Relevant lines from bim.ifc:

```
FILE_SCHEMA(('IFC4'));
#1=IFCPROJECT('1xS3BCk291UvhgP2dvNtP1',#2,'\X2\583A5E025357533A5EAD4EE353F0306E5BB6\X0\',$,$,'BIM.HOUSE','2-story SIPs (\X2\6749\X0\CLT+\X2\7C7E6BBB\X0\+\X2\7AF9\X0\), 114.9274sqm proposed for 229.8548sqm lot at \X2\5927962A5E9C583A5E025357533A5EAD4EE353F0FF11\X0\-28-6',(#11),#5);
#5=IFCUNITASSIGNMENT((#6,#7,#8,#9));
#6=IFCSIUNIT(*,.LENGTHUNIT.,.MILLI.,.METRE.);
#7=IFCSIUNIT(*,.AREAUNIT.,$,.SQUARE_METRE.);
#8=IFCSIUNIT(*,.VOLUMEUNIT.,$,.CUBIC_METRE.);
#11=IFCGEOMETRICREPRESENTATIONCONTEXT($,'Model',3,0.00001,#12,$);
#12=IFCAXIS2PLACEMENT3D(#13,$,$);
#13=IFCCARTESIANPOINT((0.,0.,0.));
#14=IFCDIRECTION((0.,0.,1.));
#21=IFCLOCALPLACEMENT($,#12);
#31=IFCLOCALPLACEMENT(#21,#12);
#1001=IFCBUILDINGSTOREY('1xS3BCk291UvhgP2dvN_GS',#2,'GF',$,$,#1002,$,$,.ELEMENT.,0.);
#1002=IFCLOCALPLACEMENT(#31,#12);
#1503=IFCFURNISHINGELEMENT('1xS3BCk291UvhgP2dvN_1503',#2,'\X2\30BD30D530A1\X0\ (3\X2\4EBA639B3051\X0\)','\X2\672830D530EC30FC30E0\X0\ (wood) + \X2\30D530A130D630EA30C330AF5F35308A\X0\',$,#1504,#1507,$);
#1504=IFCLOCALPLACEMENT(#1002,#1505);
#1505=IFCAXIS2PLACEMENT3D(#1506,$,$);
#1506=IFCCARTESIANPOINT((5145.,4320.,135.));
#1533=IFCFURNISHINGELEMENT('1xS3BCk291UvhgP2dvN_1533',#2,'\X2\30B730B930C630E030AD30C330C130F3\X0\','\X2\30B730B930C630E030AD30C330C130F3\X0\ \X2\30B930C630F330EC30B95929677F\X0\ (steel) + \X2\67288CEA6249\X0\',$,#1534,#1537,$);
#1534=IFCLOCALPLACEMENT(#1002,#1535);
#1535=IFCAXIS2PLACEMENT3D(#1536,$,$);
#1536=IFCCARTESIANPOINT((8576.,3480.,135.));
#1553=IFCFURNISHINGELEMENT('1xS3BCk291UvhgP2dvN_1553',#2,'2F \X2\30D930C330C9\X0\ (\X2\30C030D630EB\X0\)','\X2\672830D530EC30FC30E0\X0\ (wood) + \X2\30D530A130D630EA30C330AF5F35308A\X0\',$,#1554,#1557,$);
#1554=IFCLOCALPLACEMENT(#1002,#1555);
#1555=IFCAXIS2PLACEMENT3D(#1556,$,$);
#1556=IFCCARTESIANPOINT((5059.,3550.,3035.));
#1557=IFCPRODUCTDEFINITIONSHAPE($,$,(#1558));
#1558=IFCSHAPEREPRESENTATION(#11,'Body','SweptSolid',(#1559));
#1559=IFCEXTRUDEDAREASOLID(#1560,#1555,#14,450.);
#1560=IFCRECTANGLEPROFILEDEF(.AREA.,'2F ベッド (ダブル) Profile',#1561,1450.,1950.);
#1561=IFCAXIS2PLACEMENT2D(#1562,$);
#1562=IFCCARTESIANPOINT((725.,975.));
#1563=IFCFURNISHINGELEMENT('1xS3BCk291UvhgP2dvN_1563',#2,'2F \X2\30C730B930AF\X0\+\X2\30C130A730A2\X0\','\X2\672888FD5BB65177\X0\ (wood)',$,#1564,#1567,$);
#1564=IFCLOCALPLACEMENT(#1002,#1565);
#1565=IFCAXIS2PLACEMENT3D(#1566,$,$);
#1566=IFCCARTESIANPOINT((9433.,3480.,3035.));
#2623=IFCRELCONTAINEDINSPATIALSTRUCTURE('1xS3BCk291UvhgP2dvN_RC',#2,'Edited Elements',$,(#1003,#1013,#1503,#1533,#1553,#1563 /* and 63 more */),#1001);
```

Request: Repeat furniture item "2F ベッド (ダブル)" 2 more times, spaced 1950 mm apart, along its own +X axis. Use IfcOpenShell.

```python
import ifcopenshell
import ifcopenshell.api.geometry
import ifcopenshell.api.root
import ifcopenshell.util.element
import ifcopenshell.util.placement

model = ifcopenshell.open("bim.ifc")


def reuse_history(source, copy):
    """copy_class also copies each property set's owner history, people and application; keep the originals."""
    for rel in copy.IsDefinedBy:
        if rel.is_a("IfcRelDefinesByProperties") and (history := rel.RelatingPropertyDefinition.OwnerHistory):
            rel.RelatingPropertyDefinition.OwnerHistory = source.OwnerHistory
            ifcopenshell.util.element.remove_deep2(model, history)


source = model.by_guid("1xS3BCk291UvhgP2dvN_1553")
base = ifcopenshell.util.placement.get_local_placement(source.ObjectPlacement)
step = base[:3, 0] * 1950.0

for i in range(1, 3):
    copy = ifcopenshell.api.root.copy_class(model, product=source)
    copy.Representation = ifcopenshell.util.element.copy_deep(
        model, source.Representation, exclude=["IfcGeometricRepresentationContext", "IfcRepresentationMap"]
    )
    reuse_history(source, copy)
    matrix = base.copy()
    matrix[:3, 3] += i * step
    print("added at", matrix[:3, 3].round(3) + 0.0)
    ifcopenshell.api.geometry.edit_object_placement(model, product=copy, matrix=matrix, is_si=False)

model.write("bim-out.ifc")
```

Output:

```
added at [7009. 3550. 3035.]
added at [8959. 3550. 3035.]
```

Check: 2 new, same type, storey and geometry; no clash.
